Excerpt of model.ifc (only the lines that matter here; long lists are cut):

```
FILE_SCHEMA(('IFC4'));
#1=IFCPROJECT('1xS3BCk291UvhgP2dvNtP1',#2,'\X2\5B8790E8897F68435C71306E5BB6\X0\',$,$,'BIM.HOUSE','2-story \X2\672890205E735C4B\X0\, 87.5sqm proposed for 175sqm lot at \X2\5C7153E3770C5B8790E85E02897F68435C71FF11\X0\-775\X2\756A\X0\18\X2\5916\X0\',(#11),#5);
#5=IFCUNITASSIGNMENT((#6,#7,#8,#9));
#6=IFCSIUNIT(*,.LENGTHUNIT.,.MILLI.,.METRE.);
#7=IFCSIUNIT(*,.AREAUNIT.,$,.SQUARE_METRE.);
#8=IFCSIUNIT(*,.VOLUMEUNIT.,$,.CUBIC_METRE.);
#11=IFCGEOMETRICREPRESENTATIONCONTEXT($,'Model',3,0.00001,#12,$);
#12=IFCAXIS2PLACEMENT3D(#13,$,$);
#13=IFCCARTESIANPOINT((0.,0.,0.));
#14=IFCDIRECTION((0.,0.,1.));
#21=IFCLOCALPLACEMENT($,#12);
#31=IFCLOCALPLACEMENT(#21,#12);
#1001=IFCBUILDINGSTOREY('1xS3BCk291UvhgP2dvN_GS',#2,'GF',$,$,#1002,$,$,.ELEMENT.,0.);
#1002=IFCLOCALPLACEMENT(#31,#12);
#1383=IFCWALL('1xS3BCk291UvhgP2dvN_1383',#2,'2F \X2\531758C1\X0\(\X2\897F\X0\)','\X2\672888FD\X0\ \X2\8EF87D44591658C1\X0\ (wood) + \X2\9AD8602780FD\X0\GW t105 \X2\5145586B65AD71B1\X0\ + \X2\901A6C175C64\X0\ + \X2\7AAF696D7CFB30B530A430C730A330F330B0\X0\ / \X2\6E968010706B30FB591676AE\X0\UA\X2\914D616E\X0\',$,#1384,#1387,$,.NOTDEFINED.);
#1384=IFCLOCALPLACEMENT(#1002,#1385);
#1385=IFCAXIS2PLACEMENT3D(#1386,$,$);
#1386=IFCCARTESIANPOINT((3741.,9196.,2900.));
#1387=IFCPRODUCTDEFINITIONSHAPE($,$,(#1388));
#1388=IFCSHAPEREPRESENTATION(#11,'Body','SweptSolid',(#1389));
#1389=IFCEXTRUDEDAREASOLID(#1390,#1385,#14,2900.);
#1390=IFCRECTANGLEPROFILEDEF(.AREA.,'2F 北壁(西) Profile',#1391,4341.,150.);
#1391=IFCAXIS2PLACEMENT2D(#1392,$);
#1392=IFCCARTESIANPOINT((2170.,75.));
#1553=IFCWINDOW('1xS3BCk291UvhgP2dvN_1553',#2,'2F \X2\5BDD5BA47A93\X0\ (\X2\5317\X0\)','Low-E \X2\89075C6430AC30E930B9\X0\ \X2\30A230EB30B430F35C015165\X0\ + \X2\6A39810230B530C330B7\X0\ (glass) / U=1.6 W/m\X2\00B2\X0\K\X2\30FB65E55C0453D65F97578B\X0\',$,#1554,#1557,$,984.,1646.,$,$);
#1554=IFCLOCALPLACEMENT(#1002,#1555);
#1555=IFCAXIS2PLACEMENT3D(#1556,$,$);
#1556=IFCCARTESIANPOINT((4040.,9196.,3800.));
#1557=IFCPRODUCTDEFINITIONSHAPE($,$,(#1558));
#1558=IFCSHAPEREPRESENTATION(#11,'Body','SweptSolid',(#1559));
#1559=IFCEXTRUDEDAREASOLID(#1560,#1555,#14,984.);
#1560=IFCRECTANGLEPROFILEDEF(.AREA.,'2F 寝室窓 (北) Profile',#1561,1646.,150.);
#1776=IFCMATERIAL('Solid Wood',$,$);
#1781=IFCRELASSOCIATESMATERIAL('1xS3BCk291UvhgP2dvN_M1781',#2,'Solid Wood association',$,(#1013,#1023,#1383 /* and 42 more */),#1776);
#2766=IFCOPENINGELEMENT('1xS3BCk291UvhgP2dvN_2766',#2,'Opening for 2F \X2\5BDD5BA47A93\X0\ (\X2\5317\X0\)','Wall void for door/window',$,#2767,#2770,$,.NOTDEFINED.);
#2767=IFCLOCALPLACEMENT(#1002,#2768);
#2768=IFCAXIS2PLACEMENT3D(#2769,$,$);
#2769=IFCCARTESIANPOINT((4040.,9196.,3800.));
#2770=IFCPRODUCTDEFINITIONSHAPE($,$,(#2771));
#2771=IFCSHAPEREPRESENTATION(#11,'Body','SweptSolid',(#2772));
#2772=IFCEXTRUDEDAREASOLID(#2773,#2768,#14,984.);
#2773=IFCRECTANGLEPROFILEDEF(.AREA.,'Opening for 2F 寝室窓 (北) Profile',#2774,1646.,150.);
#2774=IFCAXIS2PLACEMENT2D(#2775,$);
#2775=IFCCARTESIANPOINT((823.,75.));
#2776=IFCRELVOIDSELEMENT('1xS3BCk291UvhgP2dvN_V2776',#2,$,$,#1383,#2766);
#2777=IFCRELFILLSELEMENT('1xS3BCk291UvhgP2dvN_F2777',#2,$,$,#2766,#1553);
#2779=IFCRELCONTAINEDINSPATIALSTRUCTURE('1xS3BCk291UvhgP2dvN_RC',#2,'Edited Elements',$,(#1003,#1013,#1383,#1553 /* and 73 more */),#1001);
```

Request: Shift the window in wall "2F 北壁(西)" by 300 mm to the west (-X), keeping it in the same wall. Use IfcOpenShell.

```python
import ifcopenshell
import ifcopenshell.api.geometry
import ifcopenshell.util.placement
import ifcopenshell.util.unit

model = ifcopenshell.open("model.ifc")
unit_scale = ifcopenshell.util.unit.calculate_unit_scale(model)

window = model.by_id(1553)
opening = window.FillsVoids[0].RelatingOpeningElement
wall = opening.VoidsElements[0].RelatingBuildingElement

wall_matrix = ifcopenshell.util.placement.get_local_placement(wall.ObjectPlacement)
shift = wall_matrix[:3, 0] * -0.3 / unit_scale
before = ifcopenshell.util.placement.get_local_placement(window.ObjectPlacement)[:3, 3].copy()

# The window is not placed relative to its opening, so move both.
for product in (opening, window):
    matrix = ifcopenshell.util.placement.get_local_placement(product.ObjectPlacement)
    matrix[:3, 3] += shift
    ifcopenshell.api.geometry.edit_object_placement(model, product=product, matrix=matrix, is_si=False)

after = ifcopenshell.util.placement.get_local_placement(window.ObjectPlacement)[:3, 3]
print("window moved by", (after - before).round(3) + 0.0)

model.write("model_edited.ifc")
```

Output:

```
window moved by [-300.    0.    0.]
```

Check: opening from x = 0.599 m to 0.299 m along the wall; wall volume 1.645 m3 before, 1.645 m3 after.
